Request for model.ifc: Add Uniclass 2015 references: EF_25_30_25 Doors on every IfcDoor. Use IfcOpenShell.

First a look at what the model holds.

```python
import ifcopenshell

model = ifcopenshell.open("model.ifc")
print(model.schema)
print("classifications:", [c.Name for c in model.by_type("IfcClassification")])
for ifc_class in ("IfcDoor", "IfcRoof", "IfcStair", "IfcWall", "IfcWindow"):
    print(ifc_class, len(model.by_type(ifc_class)))
```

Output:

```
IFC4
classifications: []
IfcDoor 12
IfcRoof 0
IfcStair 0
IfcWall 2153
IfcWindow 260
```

```python
import ifcopenshell
import ifcopenshell.api.classification

model = ifcopenshell.open("model.ifc")

system = ifcopenshell.api.classification.add_classification(model, classification="Uniclass 2015")

codes = {
    "IfcDoor": ("EF_25_30_25", "Doors"),
}
for ifc_class, (code, name) in codes.items():
    products = model.by_type(ifc_class)
    ifcopenshell.api.classification.add_reference(
        model, products=products, classification=system, identification=code, name=name
    )
    print(code, len(products))

model.write("model_v2.ifc")
```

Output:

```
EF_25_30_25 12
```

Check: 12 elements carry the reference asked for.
